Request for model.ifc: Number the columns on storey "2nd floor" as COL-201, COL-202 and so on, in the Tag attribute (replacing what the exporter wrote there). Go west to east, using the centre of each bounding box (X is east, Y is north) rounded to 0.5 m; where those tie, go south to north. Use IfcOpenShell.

First a look at what the model holds.

```python
import ifcopenshell
import ifcopenshell.util.element
import ifcopenshell.util.placement

model = ifcopenshell.open("model.ifc")
print(model.schema)
storey = next(s for s in model.by_type("IfcBuildingStorey") if s.Name == "2nd floor")
columns = [e for e in ifcopenshell.util.element.get_decomposition(storey) if e.is_a("IfcColumn")]
for e in sorted(columns, key=lambda e: e.id()):
    origin = ifcopenshell.util.placement.get_local_placement(e.ObjectPlacement)[:3, 3]
    print(e.id(), e.Tag, e.Name, origin.round(2) + 0.0, sep=" | ")
```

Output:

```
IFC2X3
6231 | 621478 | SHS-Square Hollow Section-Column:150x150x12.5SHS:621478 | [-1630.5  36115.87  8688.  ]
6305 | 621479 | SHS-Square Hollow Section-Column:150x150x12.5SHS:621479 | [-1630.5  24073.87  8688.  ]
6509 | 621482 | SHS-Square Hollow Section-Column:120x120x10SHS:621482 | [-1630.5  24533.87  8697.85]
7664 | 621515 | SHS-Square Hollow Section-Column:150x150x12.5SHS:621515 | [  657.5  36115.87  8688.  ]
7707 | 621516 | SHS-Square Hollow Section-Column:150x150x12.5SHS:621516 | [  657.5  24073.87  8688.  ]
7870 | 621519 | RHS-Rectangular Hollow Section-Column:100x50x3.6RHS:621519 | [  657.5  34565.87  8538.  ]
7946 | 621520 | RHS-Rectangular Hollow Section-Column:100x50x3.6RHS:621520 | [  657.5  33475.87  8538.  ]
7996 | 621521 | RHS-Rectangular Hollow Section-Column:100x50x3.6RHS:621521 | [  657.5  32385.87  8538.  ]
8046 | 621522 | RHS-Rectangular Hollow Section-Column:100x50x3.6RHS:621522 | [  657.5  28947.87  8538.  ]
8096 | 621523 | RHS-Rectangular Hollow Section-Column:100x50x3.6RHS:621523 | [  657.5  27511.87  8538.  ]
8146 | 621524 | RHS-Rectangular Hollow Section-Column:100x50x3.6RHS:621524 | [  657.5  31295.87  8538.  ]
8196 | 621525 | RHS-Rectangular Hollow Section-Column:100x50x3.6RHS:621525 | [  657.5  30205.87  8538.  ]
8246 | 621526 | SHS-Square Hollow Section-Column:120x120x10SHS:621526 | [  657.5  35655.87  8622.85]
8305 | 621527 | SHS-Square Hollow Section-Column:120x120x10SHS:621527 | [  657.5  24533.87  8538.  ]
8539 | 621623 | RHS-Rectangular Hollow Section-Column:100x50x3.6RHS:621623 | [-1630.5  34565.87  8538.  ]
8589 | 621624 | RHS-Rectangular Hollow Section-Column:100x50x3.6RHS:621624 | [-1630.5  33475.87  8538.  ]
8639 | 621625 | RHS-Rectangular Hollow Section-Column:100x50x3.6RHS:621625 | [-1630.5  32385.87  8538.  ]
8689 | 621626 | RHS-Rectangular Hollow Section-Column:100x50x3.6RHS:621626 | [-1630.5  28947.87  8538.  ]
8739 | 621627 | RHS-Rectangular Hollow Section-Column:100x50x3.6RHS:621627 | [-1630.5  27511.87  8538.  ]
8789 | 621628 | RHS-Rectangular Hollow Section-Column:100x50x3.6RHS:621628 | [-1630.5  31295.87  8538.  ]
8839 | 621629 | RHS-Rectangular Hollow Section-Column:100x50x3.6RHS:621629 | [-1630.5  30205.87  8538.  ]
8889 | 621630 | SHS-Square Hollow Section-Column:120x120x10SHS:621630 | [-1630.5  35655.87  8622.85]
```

```python
import ifcopenshell
import ifcopenshell.geom
import ifcopenshell.util.element
import ifcopenshell.util.shape

model = ifcopenshell.open("model.ifc")
settings = ifcopenshell.geom.settings()
settings.set("use-world-coords", True)


def centre(element):
    shape = ifcopenshell.geom.create_shape(settings, element)
    return ifcopenshell.util.shape.get_bbox_centroid(shape.geometry)


storey = next(s for s in model.by_type("IfcBuildingStorey") if s.Name == "2nd floor")
columns = [e for e in ifcopenshell.util.element.get_decomposition(storey) if e.is_a("IfcColumn")]

# Insertion points can sit at a corner or the storey origin, so sort by the geometry (in metres).
centres = {e: centre(e) for e in columns}
columns.sort(key=lambda e: (round(centres[e][0] / 0.5), centres[e][1]))

for i, e in enumerate(columns, start=1):
    number = f"COL-2{i:02d}"
    e.Tag = number
    print(e.id(), number)

model.write("model-out.ifc")
```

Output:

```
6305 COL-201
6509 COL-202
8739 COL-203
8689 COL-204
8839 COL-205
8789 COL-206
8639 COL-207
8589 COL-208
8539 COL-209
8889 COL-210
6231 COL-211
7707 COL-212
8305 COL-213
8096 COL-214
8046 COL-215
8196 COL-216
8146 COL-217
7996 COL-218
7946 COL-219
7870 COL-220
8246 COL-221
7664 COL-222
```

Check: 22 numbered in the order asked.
